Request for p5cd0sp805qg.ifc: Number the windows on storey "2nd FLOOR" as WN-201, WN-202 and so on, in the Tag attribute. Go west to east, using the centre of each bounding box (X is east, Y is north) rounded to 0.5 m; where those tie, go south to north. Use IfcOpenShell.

First a look at what the model holds.

```python
import ifcopenshell
import ifcopenshell.util.element
import ifcopenshell.util.placement

model = ifcopenshell.open("p5cd0sp805qg.ifc")
print(model.schema)
storey = next(s for s in model.by_type("IfcBuildingStorey") if s.Name == "2nd FLOOR")
windows = [e for e in ifcopenshell.util.element.get_decomposition(storey) if e.is_a("IfcWindow")]
for e in sorted(windows, key=lambda e: e.id()):
    origin = ifcopenshell.util.placement.get_local_placement(e.ObjectPlacement)[:3, 3]
    print(e.id(), e.Tag, e.Name, origin.round(2) + 0.0, sep=" | ")
```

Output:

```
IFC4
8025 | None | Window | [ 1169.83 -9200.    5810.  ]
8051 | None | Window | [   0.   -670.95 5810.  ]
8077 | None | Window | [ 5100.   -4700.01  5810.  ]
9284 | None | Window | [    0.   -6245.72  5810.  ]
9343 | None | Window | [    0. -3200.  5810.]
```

```python
import ifcopenshell
import ifcopenshell.geom
import ifcopenshell.util.element
import ifcopenshell.util.shape

model = ifcopenshell.open("p5cd0sp805qg.ifc")
settings = ifcopenshell.geom.settings()
settings.set("use-world-coords", True)


def centre(element):
    shape = ifcopenshell.geom.create_shape(settings, element)
    return ifcopenshell.util.shape.get_bbox_centroid(shape.geometry)


storey = next(s for s in model.by_type("IfcBuildingStorey") if s.Name == "2nd FLOOR")
windows = [e for e in ifcopenshell.util.element.get_decomposition(storey) if e.is_a("IfcWindow")]

# Insertion points can sit at a corner or the storey origin, so sort by the geometry (in metres).
centres = {e: centre(e) for e in windows}
windows.sort(key=lambda e: (round(centres[e][0] / 0.5), centres[e][1]))

for i, e in enumerate(windows, start=1):
    number = f"WN-2{i:02d}"
    e.Tag = number
    print(e.id(), number)

model.write("p5cd0sp805qg_updated.ifc")
```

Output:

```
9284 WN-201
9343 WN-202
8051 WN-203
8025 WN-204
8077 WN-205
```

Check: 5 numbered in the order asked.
